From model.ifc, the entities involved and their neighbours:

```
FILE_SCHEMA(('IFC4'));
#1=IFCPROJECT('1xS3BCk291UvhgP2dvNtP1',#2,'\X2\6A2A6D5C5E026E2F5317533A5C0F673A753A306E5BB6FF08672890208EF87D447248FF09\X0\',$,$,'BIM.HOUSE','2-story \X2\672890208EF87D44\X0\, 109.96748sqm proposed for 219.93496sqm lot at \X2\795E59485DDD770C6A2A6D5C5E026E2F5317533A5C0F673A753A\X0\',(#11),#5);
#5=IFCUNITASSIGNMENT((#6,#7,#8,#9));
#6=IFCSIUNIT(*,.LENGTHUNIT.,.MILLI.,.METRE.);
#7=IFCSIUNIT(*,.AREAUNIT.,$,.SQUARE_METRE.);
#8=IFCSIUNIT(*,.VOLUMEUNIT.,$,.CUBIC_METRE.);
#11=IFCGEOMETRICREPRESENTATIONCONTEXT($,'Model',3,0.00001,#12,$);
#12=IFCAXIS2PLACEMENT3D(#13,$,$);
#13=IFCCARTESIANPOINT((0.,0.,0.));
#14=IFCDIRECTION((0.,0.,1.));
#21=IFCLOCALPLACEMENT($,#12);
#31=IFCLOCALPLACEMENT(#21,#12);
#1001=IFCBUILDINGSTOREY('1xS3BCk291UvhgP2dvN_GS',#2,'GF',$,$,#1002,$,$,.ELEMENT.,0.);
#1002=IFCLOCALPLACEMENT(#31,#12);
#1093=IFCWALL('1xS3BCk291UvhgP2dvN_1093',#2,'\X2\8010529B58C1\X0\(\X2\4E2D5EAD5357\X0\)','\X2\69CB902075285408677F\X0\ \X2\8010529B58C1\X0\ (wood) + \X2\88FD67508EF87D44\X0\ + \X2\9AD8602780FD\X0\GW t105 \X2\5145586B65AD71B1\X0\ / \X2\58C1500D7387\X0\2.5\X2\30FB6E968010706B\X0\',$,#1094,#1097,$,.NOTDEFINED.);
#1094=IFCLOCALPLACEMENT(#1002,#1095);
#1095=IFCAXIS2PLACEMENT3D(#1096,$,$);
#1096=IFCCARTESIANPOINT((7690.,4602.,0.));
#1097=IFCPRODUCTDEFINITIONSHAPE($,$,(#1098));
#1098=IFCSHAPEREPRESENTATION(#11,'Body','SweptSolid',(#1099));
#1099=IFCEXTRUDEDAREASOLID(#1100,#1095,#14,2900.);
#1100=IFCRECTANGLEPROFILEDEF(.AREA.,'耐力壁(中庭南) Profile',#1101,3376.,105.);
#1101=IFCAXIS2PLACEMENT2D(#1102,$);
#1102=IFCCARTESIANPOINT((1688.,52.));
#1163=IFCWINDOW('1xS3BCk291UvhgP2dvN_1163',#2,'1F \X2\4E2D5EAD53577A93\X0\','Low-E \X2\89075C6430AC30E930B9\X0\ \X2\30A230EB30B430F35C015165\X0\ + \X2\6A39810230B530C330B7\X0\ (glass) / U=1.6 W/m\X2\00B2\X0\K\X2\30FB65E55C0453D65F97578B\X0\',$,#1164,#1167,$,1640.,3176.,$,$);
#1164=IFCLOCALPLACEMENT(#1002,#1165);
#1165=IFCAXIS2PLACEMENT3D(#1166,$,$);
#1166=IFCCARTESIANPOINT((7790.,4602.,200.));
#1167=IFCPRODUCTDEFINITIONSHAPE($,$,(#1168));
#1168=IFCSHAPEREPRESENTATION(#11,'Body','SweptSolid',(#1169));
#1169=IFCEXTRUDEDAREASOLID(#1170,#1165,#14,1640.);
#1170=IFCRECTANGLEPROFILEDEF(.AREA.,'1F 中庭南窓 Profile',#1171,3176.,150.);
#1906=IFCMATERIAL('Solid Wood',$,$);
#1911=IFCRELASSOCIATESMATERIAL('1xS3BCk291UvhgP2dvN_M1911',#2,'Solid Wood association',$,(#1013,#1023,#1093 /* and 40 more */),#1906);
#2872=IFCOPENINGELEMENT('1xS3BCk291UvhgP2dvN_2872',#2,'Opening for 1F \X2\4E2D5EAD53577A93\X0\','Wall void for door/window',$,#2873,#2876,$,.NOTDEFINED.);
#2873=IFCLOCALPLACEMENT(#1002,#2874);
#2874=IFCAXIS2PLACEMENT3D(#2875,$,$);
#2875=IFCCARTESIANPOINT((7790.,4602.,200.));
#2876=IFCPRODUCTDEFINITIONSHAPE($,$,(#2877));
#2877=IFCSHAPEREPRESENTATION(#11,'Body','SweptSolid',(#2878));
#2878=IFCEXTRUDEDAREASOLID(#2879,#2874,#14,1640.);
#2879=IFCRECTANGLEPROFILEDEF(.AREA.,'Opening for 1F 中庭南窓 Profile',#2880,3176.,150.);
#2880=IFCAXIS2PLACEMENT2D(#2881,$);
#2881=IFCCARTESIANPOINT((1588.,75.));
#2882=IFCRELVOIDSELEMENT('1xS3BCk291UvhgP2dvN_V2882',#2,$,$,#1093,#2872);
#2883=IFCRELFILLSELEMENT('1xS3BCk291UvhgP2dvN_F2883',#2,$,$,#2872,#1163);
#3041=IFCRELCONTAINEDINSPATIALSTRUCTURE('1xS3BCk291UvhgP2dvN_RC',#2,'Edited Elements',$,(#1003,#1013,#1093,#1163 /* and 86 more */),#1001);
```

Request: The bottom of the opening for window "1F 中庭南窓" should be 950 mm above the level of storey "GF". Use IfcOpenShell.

```python
import numpy as np
import ifcopenshell
import ifcopenshell.api.geometry
import ifcopenshell.geom
import ifcopenshell.util.element
import ifcopenshell.util.placement
import ifcopenshell.util.shape
import ifcopenshell.util.unit

model = ifcopenshell.open("model.ifc")
unit_scale = ifcopenshell.util.unit.calculate_unit_scale(model)

window = model.by_guid("1xS3BCk291UvhgP2dvN_1163")
opening = window.FillsVoids[0].RelatingOpeningElement
storey = ifcopenshell.util.element.get_container(window, ifc_class="IfcBuildingStorey")
level = ifcopenshell.util.placement.get_local_placement(storey.ObjectPlacement)[2, 3]

# The opening's origin need not be at the sill, so measure its lowest point.
shape = ifcopenshell.geom.create_shape(ifcopenshell.geom.settings(), opening)
bottom = ifcopenshell.util.shape.get_shape_bottom_elevation(shape, shape.geometry) / unit_scale
dz = level + 0.95 / unit_scale - bottom

shift = np.array([0.0, 0.0, dz])
# The window is not placed relative to its opening, so move both.
for product in (opening, window):
    matrix = ifcopenshell.util.placement.get_local_placement(product.ObjectPlacement)
    matrix[:3, 3] += shift
    ifcopenshell.api.geometry.edit_object_placement(model, product=product, matrix=matrix, is_si=False)

print(f"moved by {dz * unit_scale:+.3f} m")

model.write("model_rev.ifc")
```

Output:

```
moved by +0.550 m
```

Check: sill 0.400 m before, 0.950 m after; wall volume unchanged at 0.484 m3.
